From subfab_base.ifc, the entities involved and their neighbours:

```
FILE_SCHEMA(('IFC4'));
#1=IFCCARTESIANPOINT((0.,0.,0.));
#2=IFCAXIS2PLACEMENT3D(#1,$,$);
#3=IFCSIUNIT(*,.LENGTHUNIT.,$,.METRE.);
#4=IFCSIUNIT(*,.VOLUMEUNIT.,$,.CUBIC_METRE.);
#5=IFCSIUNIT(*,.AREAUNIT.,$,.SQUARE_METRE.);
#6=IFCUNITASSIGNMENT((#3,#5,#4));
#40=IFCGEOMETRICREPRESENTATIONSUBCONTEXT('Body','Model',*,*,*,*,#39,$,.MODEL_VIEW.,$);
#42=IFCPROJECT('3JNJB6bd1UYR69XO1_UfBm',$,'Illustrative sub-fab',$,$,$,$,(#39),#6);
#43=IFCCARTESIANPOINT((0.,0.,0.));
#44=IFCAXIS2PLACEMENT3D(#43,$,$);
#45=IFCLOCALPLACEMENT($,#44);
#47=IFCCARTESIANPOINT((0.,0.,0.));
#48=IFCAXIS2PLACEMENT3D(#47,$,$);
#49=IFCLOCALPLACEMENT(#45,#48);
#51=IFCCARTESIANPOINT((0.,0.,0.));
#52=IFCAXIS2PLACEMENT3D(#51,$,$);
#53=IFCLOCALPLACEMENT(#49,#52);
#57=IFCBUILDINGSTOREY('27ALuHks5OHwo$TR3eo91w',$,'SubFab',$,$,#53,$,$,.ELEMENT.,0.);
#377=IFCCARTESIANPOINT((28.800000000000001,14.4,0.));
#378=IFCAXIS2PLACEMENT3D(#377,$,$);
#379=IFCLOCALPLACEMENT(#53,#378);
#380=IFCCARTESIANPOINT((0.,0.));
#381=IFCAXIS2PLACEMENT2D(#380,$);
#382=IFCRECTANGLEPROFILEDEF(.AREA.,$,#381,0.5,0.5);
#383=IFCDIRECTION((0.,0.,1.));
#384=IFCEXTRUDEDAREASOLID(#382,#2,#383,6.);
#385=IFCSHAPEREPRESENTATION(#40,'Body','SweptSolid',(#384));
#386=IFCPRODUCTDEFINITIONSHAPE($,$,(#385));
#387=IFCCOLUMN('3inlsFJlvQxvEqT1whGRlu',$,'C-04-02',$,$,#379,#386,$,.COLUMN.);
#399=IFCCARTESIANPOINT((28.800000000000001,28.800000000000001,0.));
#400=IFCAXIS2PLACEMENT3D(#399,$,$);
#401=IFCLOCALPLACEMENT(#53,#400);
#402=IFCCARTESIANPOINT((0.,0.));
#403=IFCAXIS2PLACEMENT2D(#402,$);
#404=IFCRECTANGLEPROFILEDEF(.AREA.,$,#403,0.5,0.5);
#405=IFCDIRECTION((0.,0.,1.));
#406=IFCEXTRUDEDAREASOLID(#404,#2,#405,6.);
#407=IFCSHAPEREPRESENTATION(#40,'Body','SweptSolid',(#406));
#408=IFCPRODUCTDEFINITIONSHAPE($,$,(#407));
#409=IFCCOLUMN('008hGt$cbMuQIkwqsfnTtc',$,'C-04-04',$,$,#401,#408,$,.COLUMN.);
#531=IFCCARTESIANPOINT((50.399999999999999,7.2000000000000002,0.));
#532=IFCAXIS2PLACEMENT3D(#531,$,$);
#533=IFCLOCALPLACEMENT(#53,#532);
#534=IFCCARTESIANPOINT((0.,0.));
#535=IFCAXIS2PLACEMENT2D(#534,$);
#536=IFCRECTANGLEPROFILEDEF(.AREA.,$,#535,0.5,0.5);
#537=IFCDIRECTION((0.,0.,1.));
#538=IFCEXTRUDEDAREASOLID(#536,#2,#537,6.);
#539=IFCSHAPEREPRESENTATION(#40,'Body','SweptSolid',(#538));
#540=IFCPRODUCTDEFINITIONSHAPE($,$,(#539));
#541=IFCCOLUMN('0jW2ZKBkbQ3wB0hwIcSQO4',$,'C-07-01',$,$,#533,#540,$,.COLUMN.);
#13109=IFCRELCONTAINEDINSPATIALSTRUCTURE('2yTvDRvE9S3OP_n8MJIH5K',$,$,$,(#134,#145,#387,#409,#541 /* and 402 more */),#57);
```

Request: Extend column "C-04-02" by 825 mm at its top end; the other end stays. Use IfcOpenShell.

```python
import ifcopenshell
import ifcopenshell.util.representation

model = ifcopenshell.open("subfab_base.ifc")

member = model.by_guid("3inlsFJlvQxvEqT1whGRlu")
change = 0.825

# The extrusion runs towards the end named, so only its depth changes.
body = ifcopenshell.util.representation.get_representation(member, "Model", "Body")
solid = body.Items[0]
old_length = solid.Depth
solid.Depth += change

print(f"length {old_length:g} -> {solid.Depth:g}")

model.write("subfab_base_rev.ifc")
```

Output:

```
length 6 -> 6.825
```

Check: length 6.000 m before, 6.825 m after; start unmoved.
